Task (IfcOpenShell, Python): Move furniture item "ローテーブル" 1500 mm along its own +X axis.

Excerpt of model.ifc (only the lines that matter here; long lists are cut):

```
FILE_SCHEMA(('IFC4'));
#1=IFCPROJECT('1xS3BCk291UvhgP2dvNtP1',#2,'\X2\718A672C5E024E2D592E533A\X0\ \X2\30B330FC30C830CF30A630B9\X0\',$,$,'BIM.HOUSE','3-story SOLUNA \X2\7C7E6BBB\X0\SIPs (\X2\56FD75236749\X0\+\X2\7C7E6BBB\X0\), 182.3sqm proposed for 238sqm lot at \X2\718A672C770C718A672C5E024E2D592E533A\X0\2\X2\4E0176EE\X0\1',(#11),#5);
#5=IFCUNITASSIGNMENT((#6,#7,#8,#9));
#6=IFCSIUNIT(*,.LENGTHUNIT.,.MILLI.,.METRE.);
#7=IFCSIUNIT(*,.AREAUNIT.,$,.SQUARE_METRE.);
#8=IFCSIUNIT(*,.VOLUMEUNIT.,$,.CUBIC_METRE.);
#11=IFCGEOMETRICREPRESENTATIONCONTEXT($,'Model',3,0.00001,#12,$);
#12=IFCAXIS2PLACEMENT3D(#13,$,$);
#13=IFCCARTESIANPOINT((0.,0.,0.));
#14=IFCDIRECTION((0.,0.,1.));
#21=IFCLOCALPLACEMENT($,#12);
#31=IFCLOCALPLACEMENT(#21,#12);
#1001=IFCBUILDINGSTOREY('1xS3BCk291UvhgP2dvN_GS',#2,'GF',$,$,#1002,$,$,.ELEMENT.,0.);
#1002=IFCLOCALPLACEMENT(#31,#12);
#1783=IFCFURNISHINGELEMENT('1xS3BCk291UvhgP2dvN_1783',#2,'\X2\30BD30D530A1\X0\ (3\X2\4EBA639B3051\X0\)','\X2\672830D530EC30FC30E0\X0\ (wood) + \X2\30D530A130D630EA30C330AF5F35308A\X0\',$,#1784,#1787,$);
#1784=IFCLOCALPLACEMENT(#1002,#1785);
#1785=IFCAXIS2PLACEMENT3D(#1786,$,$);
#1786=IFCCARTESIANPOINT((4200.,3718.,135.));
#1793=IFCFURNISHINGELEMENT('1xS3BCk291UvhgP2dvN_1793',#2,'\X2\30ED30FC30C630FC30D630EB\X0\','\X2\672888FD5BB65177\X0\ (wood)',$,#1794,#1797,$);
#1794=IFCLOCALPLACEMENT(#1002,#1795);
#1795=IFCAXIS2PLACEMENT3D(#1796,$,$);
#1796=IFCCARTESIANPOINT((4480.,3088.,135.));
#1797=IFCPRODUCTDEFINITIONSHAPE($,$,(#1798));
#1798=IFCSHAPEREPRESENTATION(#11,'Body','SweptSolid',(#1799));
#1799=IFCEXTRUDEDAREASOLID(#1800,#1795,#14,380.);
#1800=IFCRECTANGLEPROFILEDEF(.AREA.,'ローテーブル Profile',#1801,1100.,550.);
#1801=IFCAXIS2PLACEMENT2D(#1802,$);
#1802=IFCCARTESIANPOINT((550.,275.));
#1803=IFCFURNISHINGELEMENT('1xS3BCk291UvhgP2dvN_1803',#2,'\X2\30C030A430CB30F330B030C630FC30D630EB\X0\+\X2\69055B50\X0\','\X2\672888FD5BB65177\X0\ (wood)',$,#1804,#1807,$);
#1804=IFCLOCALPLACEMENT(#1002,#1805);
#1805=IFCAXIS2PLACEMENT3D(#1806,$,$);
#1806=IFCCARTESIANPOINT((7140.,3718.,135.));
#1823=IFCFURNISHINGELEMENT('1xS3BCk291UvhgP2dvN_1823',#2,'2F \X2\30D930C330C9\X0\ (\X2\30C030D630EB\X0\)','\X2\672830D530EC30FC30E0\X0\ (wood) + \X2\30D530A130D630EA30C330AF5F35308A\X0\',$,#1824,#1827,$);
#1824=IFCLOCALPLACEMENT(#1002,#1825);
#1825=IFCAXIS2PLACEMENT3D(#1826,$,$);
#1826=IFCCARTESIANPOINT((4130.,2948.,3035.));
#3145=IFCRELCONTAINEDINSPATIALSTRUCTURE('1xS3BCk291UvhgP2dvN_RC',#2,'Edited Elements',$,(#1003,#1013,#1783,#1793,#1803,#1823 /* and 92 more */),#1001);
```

```python
import ifcopenshell
import ifcopenshell.api.geometry
import ifcopenshell.util.placement

model = ifcopenshell.open("model.ifc")

item = model.by_guid("1xS3BCk291UvhgP2dvN_1793")
matrix = ifcopenshell.util.placement.get_local_placement(item.ObjectPlacement)
matrix[:3, 3] += matrix[:3, 0] * 1500.0
ifcopenshell.api.geometry.edit_object_placement(model, product=item, matrix=matrix, is_si=False)

print(ifcopenshell.util.placement.get_local_placement(item.ObjectPlacement).round(3) + 0.0)

model.write("model_edited.ifc")
```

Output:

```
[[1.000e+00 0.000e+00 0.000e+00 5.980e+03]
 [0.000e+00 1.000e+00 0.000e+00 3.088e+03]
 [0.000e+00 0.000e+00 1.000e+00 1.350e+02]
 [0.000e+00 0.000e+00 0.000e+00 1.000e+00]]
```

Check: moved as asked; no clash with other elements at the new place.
